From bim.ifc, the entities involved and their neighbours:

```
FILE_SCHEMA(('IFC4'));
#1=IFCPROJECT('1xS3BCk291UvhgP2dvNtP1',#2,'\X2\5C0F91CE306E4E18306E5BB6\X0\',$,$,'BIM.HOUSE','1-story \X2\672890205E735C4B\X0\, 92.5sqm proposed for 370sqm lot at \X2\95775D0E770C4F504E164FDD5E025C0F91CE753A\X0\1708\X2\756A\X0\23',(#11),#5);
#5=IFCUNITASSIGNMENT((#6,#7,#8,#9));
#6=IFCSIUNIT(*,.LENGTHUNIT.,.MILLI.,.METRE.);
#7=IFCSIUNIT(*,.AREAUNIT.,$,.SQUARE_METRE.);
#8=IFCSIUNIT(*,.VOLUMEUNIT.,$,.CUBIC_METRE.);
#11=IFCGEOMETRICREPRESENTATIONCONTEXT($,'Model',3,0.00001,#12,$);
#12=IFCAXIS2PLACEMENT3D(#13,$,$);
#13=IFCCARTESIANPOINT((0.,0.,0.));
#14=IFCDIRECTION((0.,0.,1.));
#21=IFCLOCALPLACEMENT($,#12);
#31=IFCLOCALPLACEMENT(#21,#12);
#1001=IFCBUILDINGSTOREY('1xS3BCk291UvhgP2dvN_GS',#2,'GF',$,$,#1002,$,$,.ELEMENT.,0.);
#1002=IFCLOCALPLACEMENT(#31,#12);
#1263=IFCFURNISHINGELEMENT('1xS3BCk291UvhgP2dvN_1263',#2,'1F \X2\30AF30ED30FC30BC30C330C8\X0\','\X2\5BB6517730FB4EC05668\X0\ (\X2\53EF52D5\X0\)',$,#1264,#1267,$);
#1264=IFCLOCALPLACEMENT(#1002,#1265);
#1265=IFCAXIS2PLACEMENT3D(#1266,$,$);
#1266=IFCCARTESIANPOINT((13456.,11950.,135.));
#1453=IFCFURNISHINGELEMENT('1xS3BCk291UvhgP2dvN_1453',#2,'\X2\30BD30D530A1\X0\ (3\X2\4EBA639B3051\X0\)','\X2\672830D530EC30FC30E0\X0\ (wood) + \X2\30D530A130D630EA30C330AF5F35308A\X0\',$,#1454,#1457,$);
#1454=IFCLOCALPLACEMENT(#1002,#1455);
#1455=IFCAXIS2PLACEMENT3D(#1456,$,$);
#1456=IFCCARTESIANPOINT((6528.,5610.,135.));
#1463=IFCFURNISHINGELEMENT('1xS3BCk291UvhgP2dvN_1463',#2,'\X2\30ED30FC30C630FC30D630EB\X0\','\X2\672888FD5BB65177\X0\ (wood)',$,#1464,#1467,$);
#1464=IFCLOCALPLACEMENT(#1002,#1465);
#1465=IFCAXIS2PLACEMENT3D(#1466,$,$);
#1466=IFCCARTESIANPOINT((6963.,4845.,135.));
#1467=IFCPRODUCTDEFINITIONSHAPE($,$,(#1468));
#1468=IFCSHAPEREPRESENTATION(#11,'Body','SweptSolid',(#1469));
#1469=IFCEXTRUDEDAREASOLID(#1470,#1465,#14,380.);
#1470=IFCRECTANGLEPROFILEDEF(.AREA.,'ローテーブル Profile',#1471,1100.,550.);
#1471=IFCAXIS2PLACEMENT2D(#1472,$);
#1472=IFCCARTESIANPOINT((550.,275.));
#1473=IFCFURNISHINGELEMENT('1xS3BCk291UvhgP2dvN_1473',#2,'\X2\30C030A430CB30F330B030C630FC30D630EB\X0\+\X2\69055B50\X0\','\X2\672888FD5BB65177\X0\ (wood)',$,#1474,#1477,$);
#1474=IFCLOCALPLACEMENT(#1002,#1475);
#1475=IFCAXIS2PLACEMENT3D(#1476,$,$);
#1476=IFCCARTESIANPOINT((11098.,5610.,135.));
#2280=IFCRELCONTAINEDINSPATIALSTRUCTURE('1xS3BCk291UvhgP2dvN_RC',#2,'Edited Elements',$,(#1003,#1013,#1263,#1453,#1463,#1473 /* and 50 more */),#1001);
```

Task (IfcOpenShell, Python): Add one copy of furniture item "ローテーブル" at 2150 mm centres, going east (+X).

```python
import numpy as np
import ifcopenshell
import ifcopenshell.api.geometry
import ifcopenshell.api.root
import ifcopenshell.util.element
import ifcopenshell.util.placement
import ifcopenshell.util.unit

model = ifcopenshell.open("bim.ifc")
unit_scale = ifcopenshell.util.unit.calculate_unit_scale(model)


def reuse_history(source, copy):
    """copy_class also copies each property set's owner history, people and application; keep the originals."""
    for rel in copy.IsDefinedBy:
        if rel.is_a("IfcRelDefinesByProperties") and (history := rel.RelatingPropertyDefinition.OwnerHistory):
            rel.RelatingPropertyDefinition.OwnerHistory = source.OwnerHistory
            ifcopenshell.util.element.remove_deep2(model, history)


source = model.by_guid("1xS3BCk291UvhgP2dvN_1463")
base = ifcopenshell.util.placement.get_local_placement(source.ObjectPlacement)
step = np.array([1.0, 0.0, 0.0]) * 2.15 / unit_scale

for i in range(1, 2):
    copy = ifcopenshell.api.root.copy_class(model, product=source)
    copy.Representation = ifcopenshell.util.element.copy_deep(
        model, source.Representation, exclude=["IfcGeometricRepresentationContext", "IfcRepresentationMap"]
    )
    reuse_history(source, copy)
    matrix = base.copy()
    matrix[:3, 3] += i * step
    print("added at", matrix[:3, 3].round(3) + 0.0)
    ifcopenshell.api.geometry.edit_object_placement(model, product=copy, matrix=matrix, is_si=False)

model.write("bim_updated.ifc")
```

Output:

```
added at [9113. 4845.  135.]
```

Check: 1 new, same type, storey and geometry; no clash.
